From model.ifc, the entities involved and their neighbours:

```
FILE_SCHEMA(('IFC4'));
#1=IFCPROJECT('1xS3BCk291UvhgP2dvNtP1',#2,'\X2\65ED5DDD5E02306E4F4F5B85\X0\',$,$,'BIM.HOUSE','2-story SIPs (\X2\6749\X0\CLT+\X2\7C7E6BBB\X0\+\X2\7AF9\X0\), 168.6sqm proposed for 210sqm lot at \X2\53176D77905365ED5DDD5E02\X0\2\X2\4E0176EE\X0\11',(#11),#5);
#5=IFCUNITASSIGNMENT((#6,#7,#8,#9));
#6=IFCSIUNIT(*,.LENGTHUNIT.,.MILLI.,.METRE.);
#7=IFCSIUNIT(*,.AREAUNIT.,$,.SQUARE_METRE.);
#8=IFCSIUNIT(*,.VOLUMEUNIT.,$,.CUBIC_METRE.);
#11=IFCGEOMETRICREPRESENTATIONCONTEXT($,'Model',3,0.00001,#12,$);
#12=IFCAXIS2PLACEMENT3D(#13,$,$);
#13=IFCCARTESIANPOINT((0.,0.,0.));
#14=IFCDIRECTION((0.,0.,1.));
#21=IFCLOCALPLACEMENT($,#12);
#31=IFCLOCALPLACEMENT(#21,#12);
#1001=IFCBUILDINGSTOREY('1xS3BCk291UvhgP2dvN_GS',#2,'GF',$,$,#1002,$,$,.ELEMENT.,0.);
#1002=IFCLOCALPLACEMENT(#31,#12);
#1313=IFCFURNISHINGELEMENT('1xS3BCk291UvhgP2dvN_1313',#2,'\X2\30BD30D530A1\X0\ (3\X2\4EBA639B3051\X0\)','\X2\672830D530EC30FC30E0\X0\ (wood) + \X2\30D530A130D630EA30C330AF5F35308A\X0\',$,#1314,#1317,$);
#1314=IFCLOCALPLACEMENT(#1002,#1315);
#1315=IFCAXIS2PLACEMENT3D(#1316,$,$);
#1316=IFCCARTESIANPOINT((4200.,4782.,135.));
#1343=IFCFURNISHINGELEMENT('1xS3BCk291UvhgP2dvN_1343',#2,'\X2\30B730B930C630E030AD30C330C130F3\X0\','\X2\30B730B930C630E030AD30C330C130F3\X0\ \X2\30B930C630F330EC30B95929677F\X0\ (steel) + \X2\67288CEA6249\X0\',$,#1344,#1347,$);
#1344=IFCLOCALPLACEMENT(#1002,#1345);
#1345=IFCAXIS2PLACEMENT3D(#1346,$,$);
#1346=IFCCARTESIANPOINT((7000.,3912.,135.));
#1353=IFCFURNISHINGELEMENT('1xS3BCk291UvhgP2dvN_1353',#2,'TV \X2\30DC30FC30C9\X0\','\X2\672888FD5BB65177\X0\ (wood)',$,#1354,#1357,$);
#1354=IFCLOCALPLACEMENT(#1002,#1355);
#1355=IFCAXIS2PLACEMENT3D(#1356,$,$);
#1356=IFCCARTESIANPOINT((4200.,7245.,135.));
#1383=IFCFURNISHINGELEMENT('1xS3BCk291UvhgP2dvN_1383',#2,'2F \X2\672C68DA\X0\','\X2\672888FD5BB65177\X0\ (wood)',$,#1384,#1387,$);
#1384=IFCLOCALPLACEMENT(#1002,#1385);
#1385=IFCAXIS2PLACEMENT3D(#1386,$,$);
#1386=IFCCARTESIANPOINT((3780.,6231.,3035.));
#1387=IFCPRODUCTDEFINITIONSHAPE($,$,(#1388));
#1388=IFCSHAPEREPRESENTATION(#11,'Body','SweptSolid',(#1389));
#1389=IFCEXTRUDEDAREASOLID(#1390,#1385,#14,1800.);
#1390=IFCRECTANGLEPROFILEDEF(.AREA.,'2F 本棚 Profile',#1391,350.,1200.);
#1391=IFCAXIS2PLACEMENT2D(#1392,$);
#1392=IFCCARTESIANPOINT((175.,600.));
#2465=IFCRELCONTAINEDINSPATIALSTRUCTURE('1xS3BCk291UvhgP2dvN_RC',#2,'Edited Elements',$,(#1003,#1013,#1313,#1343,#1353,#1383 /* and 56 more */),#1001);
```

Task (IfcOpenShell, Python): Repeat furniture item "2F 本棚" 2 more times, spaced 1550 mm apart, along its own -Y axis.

```python
import ifcopenshell
import ifcopenshell.api.geometry
import ifcopenshell.api.root
import ifcopenshell.util.element
import ifcopenshell.util.placement

model = ifcopenshell.open("model.ifc")


def reuse_history(source, copy):
    """copy_class also copies each property set's owner history, people and application; keep the originals."""
    for rel in copy.IsDefinedBy:
        if rel.is_a("IfcRelDefinesByProperties") and (history := rel.RelatingPropertyDefinition.OwnerHistory):
            rel.RelatingPropertyDefinition.OwnerHistory = source.OwnerHistory
            ifcopenshell.util.element.remove_deep2(model, history)


source = model.by_guid("1xS3BCk291UvhgP2dvN_1383")
base = ifcopenshell.util.placement.get_local_placement(source.ObjectPlacement)
step = -base[:3, 1] * 1550.0

for i in range(1, 3):
    copy = ifcopenshell.api.root.copy_class(model, product=source)
    copy.Representation = ifcopenshell.util.element.copy_deep(
        model, source.Representation, exclude=["IfcGeometricRepresentationContext", "IfcRepresentationMap"]
    )
    reuse_history(source, copy)
    matrix = base.copy()
    matrix[:3, 3] += i * step
    print("added at", matrix[:3, 3].round(3) + 0.0)
    ifcopenshell.api.geometry.edit_object_placement(model, product=copy, matrix=matrix, is_si=False)

model.write("model_updated.ifc")
```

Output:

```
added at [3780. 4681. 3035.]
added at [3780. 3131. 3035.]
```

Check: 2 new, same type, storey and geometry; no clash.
